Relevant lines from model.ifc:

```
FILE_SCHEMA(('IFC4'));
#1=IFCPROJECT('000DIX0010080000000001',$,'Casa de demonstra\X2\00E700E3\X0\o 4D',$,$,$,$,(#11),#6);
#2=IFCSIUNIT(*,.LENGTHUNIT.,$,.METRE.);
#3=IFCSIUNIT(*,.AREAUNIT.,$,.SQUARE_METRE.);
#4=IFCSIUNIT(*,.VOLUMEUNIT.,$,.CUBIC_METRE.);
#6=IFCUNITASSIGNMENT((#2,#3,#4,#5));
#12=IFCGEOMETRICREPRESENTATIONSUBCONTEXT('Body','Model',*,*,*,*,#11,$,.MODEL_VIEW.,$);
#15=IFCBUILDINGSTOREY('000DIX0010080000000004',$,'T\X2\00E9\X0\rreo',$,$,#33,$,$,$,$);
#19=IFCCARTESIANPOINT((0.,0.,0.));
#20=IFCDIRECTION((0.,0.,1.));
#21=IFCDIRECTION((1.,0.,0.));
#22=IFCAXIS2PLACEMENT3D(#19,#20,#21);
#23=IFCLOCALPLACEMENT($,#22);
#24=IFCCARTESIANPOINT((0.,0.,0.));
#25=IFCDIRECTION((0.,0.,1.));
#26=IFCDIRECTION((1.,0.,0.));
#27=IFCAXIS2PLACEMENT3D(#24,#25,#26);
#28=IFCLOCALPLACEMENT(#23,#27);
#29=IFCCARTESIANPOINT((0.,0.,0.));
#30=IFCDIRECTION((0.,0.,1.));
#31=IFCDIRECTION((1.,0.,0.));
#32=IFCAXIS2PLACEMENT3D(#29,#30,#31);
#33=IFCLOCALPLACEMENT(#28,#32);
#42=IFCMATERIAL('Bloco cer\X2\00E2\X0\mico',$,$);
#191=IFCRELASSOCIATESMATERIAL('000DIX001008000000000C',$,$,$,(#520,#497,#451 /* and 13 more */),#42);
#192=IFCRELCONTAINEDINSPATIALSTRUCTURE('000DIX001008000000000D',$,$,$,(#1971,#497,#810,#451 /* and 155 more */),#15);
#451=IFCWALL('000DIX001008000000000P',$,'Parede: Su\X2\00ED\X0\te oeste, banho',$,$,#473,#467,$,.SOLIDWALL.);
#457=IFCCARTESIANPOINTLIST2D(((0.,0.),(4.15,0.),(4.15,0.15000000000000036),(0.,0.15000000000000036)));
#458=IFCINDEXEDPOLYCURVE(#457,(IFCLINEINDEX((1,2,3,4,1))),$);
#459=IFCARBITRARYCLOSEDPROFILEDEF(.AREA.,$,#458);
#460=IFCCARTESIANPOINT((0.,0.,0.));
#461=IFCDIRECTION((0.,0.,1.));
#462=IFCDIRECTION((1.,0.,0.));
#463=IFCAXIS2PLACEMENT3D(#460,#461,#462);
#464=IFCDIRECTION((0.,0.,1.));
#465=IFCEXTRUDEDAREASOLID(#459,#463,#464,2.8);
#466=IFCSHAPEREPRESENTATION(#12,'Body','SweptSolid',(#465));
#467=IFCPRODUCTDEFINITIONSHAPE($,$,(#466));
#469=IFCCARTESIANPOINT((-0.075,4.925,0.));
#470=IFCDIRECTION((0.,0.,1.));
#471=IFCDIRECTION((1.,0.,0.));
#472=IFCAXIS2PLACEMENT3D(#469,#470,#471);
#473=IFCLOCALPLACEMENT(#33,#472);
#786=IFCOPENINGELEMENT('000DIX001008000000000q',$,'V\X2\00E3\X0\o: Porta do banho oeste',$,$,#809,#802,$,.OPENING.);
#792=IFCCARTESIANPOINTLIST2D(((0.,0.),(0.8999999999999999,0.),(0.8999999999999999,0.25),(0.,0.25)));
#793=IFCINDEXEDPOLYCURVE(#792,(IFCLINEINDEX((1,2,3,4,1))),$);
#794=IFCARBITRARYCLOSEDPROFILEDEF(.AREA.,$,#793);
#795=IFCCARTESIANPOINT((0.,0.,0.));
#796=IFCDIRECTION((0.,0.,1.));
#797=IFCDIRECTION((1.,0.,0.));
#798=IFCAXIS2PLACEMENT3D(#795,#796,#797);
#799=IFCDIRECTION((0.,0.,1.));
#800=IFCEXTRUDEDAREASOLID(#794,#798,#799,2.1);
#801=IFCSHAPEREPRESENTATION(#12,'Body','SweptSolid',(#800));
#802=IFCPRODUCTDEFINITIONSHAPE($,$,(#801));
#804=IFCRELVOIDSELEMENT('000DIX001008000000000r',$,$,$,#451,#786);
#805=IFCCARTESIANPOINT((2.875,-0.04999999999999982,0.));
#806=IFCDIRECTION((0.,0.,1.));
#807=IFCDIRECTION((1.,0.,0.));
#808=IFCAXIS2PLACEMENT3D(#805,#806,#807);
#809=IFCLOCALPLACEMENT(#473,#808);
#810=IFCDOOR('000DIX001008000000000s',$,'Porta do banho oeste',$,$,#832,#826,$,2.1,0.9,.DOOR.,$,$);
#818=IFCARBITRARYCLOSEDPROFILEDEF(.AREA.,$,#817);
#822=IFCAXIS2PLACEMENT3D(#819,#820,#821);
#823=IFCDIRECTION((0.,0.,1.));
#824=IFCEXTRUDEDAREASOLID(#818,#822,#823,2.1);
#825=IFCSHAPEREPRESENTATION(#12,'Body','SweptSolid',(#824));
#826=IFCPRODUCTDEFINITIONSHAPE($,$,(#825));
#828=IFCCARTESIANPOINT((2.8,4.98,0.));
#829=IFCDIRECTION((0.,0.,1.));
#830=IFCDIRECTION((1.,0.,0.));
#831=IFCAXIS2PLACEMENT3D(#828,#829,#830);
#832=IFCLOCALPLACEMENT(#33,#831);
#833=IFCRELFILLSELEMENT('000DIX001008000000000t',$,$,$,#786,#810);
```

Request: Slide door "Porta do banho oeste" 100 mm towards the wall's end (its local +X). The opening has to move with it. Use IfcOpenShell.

```python
import ifcopenshell
import ifcopenshell.api.geometry
import ifcopenshell.util.placement

model = ifcopenshell.open("model.ifc")

door = model.by_id(810)
opening = door.FillsVoids[0].RelatingOpeningElement
wall = opening.VoidsElements[0].RelatingBuildingElement

wall_matrix = ifcopenshell.util.placement.get_local_placement(wall.ObjectPlacement)
shift = wall_matrix[:3, 0] * 0.1
before = ifcopenshell.util.placement.get_local_placement(door.ObjectPlacement)[:3, 3].copy()

# The door is not placed relative to its opening, so move both.
for product in (opening, door):
    matrix = ifcopenshell.util.placement.get_local_placement(product.ObjectPlacement)
    matrix[:3, 3] += shift
    ifcopenshell.api.geometry.edit_object_placement(model, product=product, matrix=matrix, is_si=False)

after = ifcopenshell.util.placement.get_local_placement(door.ObjectPlacement)[:3, 3]
print("door moved by", (after - before).round(3) + 0.0)

model.write("model_updated.ifc")
```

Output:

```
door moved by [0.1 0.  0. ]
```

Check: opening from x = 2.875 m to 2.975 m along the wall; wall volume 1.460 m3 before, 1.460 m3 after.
